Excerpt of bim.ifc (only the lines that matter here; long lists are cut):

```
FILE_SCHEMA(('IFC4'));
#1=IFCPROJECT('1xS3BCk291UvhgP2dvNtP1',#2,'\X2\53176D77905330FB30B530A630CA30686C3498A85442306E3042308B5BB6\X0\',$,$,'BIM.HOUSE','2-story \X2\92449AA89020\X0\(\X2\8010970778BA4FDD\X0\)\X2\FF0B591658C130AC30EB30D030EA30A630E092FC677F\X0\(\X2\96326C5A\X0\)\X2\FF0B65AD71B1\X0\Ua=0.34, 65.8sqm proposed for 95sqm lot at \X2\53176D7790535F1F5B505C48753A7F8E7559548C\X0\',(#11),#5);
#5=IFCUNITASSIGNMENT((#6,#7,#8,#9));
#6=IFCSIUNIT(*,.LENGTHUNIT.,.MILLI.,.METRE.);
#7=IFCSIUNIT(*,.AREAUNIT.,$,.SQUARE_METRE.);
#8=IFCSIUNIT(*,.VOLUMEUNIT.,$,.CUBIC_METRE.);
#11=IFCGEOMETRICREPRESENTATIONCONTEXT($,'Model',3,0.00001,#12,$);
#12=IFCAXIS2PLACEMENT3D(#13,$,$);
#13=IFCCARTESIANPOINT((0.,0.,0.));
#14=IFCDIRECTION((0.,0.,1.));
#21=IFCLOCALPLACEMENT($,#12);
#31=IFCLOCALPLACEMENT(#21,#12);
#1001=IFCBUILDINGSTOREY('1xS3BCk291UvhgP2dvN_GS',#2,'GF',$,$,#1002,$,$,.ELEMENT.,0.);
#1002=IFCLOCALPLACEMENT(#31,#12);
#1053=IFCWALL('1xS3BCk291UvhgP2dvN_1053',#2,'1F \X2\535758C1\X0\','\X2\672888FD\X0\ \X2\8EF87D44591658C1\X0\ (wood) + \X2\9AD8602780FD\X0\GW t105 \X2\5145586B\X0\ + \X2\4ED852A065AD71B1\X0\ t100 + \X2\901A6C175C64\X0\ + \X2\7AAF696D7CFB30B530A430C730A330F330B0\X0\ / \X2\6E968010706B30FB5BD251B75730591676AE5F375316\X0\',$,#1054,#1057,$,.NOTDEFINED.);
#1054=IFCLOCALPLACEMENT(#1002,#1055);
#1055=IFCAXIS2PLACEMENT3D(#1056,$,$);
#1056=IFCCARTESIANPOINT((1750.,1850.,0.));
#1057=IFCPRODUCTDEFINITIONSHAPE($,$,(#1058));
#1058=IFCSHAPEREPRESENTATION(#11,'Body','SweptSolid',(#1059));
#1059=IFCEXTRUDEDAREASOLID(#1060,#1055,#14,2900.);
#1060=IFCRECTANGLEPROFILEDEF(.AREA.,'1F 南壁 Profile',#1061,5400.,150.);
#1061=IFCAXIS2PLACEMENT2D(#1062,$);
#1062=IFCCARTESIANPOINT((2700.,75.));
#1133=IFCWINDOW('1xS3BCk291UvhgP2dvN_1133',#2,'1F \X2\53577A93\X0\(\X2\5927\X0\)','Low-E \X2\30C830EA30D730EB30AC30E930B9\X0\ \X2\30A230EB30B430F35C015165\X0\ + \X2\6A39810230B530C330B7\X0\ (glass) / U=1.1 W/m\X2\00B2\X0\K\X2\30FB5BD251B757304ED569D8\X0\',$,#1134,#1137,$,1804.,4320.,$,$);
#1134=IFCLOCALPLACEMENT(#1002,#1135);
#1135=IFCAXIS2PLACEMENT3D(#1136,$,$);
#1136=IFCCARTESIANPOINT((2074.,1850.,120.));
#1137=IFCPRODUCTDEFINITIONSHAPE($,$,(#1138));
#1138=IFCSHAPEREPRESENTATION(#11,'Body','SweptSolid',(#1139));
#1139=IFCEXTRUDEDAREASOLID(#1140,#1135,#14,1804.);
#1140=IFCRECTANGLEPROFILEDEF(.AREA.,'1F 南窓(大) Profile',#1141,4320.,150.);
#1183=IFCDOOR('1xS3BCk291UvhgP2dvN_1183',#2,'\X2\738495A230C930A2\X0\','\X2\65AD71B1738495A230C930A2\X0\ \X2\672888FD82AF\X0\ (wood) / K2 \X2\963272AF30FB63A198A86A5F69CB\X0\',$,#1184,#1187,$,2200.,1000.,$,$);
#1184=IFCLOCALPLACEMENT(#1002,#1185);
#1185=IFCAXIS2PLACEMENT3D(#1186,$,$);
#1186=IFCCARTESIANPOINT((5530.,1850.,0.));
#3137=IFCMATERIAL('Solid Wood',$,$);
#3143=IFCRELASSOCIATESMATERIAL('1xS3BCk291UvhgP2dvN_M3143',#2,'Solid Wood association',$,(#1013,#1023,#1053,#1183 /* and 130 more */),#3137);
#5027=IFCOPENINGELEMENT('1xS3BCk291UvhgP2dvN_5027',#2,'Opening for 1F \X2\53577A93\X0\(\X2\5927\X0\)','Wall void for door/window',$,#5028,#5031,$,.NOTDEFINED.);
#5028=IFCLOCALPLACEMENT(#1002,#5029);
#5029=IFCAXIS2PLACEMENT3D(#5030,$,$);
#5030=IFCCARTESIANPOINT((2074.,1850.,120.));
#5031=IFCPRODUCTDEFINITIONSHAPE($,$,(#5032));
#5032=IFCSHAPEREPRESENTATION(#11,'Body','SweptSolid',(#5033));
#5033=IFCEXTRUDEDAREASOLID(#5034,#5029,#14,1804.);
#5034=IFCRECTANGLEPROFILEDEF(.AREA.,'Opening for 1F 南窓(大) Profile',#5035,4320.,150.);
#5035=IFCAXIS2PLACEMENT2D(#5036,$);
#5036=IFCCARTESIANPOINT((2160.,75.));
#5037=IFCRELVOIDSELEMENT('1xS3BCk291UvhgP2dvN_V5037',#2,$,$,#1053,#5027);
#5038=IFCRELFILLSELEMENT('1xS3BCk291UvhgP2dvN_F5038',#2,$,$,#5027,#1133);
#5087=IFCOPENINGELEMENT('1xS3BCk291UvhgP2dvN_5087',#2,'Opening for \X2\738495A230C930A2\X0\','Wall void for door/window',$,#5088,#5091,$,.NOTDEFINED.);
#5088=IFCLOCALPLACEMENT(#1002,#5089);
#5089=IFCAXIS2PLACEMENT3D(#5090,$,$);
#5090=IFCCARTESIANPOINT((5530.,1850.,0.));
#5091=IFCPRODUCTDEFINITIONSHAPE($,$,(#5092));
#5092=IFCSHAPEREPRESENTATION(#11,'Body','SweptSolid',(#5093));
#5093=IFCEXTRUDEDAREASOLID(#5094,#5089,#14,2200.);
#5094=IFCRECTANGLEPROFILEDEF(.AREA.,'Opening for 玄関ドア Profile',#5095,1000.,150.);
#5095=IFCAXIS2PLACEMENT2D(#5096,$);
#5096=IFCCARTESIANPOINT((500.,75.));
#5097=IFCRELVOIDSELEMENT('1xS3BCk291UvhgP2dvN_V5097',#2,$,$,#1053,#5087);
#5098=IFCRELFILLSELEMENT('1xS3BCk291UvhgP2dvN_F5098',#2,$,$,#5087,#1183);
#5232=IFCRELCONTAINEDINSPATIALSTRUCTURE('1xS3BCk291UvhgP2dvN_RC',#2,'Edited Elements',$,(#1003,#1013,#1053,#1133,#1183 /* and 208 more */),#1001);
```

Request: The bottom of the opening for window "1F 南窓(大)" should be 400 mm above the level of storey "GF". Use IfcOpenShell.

```python
import numpy as np
import ifcopenshell
import ifcopenshell.api.geometry
import ifcopenshell.geom
import ifcopenshell.util.element
import ifcopenshell.util.placement
import ifcopenshell.util.shape
import ifcopenshell.util.unit

model = ifcopenshell.open("bim.ifc")
unit_scale = ifcopenshell.util.unit.calculate_unit_scale(model)

window = model.by_guid("1xS3BCk291UvhgP2dvN_1133")
opening = window.FillsVoids[0].RelatingOpeningElement
storey = ifcopenshell.util.element.get_container(window, ifc_class="IfcBuildingStorey")
level = ifcopenshell.util.placement.get_local_placement(storey.ObjectPlacement)[2, 3]

# The opening's origin need not be at the sill, so measure its lowest point.
shape = ifcopenshell.geom.create_shape(ifcopenshell.geom.settings(), opening)
bottom = ifcopenshell.util.shape.get_shape_bottom_elevation(shape, shape.geometry) / unit_scale
dz = level + 400.0 - bottom

shift = np.array([0.0, 0.0, dz])
# The window is not placed relative to its opening, so move both.
for product in (opening, window):
    matrix = ifcopenshell.util.placement.get_local_placement(product.ObjectPlacement)
    matrix[:3, 3] += shift
    ifcopenshell.api.geometry.edit_object_placement(model, product=product, matrix=matrix, is_si=False)

print(f"moved by {dz * unit_scale:+.3f} m")

model.write("bim_edited.ifc")
```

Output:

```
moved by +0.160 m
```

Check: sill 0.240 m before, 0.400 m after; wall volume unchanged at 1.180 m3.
